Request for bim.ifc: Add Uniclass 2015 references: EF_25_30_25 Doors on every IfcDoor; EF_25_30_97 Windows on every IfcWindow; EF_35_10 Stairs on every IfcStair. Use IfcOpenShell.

First a look at what the model holds.

```python
import ifcopenshell

model = ifcopenshell.open("bim.ifc")
print(model.schema)
print("classifications:", [c.Name for c in model.by_type("IfcClassification")])
for ifc_class in ("IfcDoor", "IfcRoof", "IfcStair", "IfcWall", "IfcWindow"):
    print(ifc_class, len(model.by_type(ifc_class)))
```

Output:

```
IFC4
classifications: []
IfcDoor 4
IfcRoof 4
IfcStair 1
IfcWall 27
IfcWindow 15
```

```python
import ifcopenshell
import ifcopenshell.api.classification

model = ifcopenshell.open("bim.ifc")

system = ifcopenshell.api.classification.add_classification(model, classification="Uniclass 2015")

codes = {
    "IfcDoor": ("EF_25_30_25", "Doors"),
    "IfcWindow": ("EF_25_30_97", "Windows"),
    "IfcStair": ("EF_35_10", "Stairs"),
}
for ifc_class, (code, name) in codes.items():
    products = model.by_type(ifc_class)
    ifcopenshell.api.classification.add_reference(
        model, products=products, classification=system, identification=code, name=name
    )
    print(code, len(products))

model.write("bim_edited.ifc")
```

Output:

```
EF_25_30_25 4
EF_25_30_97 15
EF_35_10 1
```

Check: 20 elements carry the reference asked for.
